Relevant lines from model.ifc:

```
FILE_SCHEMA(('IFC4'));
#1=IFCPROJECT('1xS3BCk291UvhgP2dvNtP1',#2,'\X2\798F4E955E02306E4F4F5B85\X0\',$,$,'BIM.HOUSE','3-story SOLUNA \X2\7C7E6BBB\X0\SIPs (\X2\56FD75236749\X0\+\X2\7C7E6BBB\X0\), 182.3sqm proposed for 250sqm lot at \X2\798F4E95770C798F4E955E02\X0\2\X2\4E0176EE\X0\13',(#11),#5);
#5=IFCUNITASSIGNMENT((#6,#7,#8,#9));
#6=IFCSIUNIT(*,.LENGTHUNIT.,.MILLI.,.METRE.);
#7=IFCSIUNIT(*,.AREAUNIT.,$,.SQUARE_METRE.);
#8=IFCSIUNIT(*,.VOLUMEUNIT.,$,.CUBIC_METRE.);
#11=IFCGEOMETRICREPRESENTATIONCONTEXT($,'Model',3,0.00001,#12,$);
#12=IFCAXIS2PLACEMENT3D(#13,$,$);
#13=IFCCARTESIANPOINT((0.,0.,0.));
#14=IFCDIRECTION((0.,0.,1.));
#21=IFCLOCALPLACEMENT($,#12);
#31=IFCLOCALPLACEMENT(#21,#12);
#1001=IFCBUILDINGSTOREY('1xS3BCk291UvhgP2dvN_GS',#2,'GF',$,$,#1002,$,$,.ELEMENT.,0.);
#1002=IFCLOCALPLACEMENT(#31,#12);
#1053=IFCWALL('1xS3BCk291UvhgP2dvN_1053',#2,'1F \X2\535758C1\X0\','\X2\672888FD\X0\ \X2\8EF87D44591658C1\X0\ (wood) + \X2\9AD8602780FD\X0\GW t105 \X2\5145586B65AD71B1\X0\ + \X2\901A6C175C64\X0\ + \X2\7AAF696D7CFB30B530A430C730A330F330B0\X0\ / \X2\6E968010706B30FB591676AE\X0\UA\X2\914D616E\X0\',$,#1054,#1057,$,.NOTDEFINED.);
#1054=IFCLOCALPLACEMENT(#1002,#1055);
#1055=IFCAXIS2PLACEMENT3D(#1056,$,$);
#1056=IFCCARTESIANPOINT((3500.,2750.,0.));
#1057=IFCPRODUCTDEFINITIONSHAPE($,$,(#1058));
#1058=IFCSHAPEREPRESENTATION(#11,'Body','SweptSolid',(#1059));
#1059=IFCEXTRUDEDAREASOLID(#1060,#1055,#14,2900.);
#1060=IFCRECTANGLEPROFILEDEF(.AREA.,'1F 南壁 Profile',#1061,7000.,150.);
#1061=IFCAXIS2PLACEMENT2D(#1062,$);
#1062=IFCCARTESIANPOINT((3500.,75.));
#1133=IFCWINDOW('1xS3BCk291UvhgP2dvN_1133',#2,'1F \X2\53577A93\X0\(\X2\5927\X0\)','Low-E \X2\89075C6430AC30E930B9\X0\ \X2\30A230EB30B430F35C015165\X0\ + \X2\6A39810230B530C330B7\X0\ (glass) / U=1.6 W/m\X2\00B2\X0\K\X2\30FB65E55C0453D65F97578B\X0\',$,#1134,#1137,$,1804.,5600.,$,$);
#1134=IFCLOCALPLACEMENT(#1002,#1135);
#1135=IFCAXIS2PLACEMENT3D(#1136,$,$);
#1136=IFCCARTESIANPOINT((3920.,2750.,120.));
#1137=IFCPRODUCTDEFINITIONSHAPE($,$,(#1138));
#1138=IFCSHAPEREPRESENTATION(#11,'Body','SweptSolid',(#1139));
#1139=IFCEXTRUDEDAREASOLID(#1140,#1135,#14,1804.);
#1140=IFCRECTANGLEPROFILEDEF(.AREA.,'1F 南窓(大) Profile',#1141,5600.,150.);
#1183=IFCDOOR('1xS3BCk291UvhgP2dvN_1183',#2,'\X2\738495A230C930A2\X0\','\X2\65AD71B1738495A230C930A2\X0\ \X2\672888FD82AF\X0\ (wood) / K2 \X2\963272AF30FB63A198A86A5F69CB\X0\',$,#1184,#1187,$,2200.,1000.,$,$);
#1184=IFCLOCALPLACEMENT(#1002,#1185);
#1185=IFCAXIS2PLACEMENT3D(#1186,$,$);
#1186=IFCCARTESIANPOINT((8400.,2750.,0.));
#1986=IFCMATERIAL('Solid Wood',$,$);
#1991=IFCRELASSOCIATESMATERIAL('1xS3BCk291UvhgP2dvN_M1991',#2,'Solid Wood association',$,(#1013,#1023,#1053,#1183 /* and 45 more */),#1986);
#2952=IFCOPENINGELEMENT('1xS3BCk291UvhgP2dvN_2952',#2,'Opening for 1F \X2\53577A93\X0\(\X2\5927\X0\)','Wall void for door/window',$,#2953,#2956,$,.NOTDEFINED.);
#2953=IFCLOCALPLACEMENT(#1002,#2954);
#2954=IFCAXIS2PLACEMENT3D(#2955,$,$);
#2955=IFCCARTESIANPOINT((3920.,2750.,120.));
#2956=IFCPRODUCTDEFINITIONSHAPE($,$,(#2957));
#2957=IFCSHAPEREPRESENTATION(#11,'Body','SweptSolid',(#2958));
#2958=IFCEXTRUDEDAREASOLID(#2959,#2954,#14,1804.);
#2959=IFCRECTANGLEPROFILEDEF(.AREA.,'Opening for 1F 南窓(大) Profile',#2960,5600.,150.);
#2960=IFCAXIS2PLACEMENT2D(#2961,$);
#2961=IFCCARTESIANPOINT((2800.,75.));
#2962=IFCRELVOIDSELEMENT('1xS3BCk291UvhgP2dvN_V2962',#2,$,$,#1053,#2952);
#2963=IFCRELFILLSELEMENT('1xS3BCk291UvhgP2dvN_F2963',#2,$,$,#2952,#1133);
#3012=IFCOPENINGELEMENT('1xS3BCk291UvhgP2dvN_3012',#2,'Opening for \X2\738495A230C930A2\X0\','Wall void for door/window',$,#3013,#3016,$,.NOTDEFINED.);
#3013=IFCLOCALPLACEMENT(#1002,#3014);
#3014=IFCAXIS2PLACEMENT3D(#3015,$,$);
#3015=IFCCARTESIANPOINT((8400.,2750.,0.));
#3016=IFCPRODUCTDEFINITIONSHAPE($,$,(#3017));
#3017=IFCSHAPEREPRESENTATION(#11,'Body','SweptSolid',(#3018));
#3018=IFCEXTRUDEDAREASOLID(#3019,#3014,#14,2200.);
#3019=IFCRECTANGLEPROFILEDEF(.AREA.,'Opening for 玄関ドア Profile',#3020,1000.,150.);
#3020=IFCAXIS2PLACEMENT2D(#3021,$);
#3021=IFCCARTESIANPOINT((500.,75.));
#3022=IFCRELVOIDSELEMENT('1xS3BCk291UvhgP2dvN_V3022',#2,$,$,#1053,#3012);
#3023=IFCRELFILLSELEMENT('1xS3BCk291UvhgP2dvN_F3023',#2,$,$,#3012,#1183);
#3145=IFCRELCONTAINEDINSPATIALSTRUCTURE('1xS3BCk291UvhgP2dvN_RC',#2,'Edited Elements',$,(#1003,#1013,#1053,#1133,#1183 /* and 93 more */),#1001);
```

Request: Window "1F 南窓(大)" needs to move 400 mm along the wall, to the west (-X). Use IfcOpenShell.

```python
import ifcopenshell
import ifcopenshell.api.geometry
import ifcopenshell.util.placement

model = ifcopenshell.open("model.ifc")

window = model.by_guid("1xS3BCk291UvhgP2dvN_1133")
opening = window.FillsVoids[0].RelatingOpeningElement
wall = opening.VoidsElements[0].RelatingBuildingElement

wall_matrix = ifcopenshell.util.placement.get_local_placement(wall.ObjectPlacement)
shift = wall_matrix[:3, 0] * -400.0
before = ifcopenshell.util.placement.get_local_placement(window.ObjectPlacement)[:3, 3].copy()

# The window is not placed relative to its opening, so move both.
for product in (opening, window):
    matrix = ifcopenshell.util.placement.get_local_placement(product.ObjectPlacement)
    matrix[:3, 3] += shift
    ifcopenshell.api.geometry.edit_object_placement(model, product=product, matrix=matrix, is_si=False)

after = ifcopenshell.util.placement.get_local_placement(window.ObjectPlacement)[:3, 3]
print("window moved by", (after - before).round(3) + 0.0)

model.write("model-out.ifc")
```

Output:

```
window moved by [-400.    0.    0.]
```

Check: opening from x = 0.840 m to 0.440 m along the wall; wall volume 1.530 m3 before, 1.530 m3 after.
